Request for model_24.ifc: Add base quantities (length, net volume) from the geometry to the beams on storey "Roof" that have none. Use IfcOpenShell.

First a look at what the model holds.

```python
import ifcopenshell
import ifcopenshell.util.element
import ifcopenshell.util.unit

model = ifcopenshell.open("model_24.ifc")
print(model.schema)
for unit_type in ("LENGTHUNIT", "AREAUNIT", "VOLUMEUNIT"):
    print(unit_type, ifcopenshell.util.unit.calculate_unit_scale(model, unit_type))
storey = next(s for s in model.by_type("IfcBuildingStorey") if s.Name == "Roof")
beams = [e for e in ifcopenshell.util.element.get_decomposition(storey) if e.is_a("IfcBeam")]
for e in sorted(beams, key=lambda e: e.id()):
    print(e.id(), e.is_a(), e.Name, list(ifcopenshell.util.element.get_psets(e, qtos_only=True)), sep=" | ")
```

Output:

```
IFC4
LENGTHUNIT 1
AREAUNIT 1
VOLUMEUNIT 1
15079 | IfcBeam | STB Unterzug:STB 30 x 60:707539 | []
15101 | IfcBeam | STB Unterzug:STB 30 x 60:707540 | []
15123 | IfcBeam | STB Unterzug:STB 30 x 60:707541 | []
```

```python
import ifcopenshell
import ifcopenshell.api.pset
import ifcopenshell.geom
import ifcopenshell.util.element
import ifcopenshell.util.shape
import ifcopenshell.util.unit

model = ifcopenshell.open("model_24.ifc")
unit_scale = ifcopenshell.util.unit.calculate_unit_scale(model)
volume_scale = ifcopenshell.util.unit.calculate_unit_scale(model, "VOLUMEUNIT")
settings = ifcopenshell.geom.settings()

storey = next(s for s in model.by_type("IfcBuildingStorey") if s.Name == "Roof")
beams = [e for e in ifcopenshell.util.element.get_decomposition(storey) if e.is_a("IfcBeam")]

for e in sorted(beams, key=lambda e: e.id()):
    if ifcopenshell.util.element.get_psets(e, qtos_only=True, should_inherit=False):
        continue
    # Geometry comes back in metres, in the element's own axes.
    shape = ifcopenshell.geom.create_shape(settings, e)
    values = {
        "Length": ifcopenshell.util.shape.get_max_xyz(shape.geometry) / unit_scale,
        "NetVolume": ifcopenshell.util.shape.get_volume(shape.geometry) / volume_scale,
    }
    qto = ifcopenshell.api.pset.add_qto(model, product=e, name="Qto_BeamBaseQuantities")
    ifcopenshell.api.pset.edit_qto(model, qto=qto, properties=values)
    print(e.id(), {k: round(v, 3) for k, v in values.items()})

model.write("model_24_edited.ifc")
```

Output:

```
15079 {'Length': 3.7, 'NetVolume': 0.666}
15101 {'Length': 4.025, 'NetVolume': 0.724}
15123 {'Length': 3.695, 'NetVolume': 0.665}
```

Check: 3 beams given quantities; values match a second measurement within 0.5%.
